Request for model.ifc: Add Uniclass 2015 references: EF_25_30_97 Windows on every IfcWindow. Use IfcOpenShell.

First a look at what the model holds.

```python
import ifcopenshell

model = ifcopenshell.open("model.ifc")
print(model.schema)
print("classifications:", [c.Name for c in model.by_type("IfcClassification")])
for ifc_class in ("IfcDoor", "IfcRoof", "IfcStair", "IfcWall", "IfcWindow"):
    print(ifc_class, len(model.by_type(ifc_class)))
```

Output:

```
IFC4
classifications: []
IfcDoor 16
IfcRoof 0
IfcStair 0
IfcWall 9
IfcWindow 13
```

```python
import ifcopenshell
import ifcopenshell.api.classification

model = ifcopenshell.open("model.ifc")

system = ifcopenshell.api.classification.add_classification(model, classification="Uniclass 2015")

codes = {
    "IfcWindow": ("EF_25_30_97", "Windows"),
}
for ifc_class, (code, name) in codes.items():
    products = model.by_type(ifc_class)
    ifcopenshell.api.classification.add_reference(
        model, products=products, classification=system, identification=code, name=name
    )
    print(code, len(products))

model.write("model-out.ifc")
```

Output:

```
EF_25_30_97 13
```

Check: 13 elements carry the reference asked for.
